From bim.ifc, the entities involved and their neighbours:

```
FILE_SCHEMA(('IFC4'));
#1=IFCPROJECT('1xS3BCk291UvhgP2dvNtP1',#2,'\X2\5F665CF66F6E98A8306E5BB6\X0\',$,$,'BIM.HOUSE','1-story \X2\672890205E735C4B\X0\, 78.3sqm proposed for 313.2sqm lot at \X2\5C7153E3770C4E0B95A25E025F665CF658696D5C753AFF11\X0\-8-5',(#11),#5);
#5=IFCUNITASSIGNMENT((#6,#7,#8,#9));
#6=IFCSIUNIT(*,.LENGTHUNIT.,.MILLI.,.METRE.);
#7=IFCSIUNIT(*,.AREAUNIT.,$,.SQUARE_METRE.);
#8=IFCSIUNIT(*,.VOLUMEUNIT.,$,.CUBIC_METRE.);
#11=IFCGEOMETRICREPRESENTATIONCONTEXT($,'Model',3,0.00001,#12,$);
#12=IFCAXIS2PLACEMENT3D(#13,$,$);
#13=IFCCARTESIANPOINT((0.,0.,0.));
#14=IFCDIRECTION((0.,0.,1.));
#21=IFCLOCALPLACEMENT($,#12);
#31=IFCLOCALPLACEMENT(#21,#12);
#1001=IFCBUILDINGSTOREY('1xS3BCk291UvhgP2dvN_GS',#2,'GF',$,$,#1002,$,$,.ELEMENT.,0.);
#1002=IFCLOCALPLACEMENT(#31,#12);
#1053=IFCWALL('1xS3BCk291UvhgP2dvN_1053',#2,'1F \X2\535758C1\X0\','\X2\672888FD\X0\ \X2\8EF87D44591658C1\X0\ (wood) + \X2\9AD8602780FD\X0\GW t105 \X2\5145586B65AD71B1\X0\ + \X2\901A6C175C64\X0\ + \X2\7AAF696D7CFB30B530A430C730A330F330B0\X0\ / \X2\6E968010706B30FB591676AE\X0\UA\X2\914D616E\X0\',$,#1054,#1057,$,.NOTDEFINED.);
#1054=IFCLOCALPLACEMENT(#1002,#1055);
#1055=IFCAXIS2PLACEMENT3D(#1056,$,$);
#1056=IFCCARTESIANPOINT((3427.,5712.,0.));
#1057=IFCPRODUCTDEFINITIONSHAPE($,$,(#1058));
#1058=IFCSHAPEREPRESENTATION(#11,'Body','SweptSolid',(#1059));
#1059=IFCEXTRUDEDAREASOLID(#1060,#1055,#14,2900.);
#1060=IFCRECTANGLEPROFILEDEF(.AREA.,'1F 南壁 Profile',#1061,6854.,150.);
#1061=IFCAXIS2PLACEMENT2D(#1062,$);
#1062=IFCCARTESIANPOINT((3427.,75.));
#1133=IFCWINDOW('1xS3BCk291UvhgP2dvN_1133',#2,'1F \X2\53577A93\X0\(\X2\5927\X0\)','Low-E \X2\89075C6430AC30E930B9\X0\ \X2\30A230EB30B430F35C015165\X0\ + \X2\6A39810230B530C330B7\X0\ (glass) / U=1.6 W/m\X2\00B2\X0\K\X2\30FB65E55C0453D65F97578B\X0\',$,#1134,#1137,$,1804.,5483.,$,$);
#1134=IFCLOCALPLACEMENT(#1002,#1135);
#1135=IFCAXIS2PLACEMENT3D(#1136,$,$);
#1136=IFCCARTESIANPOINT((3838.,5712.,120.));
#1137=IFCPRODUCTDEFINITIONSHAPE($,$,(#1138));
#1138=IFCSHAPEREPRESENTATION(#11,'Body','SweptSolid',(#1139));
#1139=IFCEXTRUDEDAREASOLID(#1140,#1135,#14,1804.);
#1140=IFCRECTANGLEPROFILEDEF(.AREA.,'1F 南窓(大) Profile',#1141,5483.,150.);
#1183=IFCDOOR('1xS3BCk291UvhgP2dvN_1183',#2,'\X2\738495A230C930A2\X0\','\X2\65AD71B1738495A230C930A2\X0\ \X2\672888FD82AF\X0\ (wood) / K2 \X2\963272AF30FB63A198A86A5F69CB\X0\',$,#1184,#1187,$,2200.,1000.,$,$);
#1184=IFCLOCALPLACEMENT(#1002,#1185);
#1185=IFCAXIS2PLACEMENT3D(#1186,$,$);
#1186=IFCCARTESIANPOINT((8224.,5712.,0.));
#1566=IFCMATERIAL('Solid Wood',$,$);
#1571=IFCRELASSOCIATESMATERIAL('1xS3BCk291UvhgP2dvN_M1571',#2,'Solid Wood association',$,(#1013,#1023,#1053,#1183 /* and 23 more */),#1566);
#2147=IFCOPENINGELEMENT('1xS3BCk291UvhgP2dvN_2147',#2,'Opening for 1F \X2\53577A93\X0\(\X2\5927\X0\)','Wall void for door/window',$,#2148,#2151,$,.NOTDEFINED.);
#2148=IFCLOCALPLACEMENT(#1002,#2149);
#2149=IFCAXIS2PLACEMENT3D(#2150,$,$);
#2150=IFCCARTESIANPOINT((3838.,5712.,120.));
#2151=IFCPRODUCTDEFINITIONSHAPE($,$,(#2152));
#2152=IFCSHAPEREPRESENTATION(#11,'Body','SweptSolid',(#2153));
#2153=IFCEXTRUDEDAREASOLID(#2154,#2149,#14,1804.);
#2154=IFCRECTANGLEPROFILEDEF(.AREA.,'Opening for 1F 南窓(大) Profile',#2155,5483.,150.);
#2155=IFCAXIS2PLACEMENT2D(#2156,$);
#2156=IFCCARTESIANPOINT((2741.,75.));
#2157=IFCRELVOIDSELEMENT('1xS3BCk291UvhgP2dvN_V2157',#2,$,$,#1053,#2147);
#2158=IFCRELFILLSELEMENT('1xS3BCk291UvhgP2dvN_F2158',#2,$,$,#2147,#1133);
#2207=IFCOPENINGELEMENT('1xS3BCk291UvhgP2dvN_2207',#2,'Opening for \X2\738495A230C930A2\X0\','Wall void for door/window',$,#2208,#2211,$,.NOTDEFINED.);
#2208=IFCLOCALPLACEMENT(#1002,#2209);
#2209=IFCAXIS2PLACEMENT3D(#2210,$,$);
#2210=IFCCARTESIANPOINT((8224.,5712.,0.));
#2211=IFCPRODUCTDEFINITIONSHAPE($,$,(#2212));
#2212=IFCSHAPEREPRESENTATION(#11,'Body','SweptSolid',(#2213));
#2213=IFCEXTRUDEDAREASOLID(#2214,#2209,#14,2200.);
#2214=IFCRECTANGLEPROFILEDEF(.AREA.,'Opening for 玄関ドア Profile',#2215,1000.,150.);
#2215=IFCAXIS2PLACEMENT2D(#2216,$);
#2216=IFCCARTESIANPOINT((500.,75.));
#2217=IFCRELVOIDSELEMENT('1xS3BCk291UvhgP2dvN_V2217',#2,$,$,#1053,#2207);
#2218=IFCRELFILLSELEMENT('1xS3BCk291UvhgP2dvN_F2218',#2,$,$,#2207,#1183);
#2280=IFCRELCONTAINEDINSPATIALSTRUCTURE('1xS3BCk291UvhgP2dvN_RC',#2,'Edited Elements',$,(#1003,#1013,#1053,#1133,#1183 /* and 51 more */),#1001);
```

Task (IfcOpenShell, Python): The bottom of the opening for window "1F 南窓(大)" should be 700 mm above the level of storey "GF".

```python
import numpy as np
import ifcopenshell
import ifcopenshell.api.geometry
import ifcopenshell.geom
import ifcopenshell.util.element
import ifcopenshell.util.placement
import ifcopenshell.util.shape
import ifcopenshell.util.unit

model = ifcopenshell.open("bim.ifc")
unit_scale = ifcopenshell.util.unit.calculate_unit_scale(model)

window = model.by_guid("1xS3BCk291UvhgP2dvN_1133")
opening = window.FillsVoids[0].RelatingOpeningElement
storey = ifcopenshell.util.element.get_container(window, ifc_class="IfcBuildingStorey")
level = ifcopenshell.util.placement.get_local_placement(storey.ObjectPlacement)[2, 3]

# The opening's origin need not be at the sill, so measure its lowest point.
shape = ifcopenshell.geom.create_shape(ifcopenshell.geom.settings(), opening)
bottom = ifcopenshell.util.shape.get_shape_bottom_elevation(shape, shape.geometry) / unit_scale
dz = level + 700.0 - bottom

shift = np.array([0.0, 0.0, dz])
# The window is not placed relative to its opening, so move both.
for product in (opening, window):
    matrix = ifcopenshell.util.placement.get_local_placement(product.ObjectPlacement)
    matrix[:3, 3] += shift
    ifcopenshell.api.geometry.edit_object_placement(model, product=product, matrix=matrix, is_si=False)

print(f"moved by {dz * unit_scale:+.3f} m")

model.write("bim_rev.ifc")
```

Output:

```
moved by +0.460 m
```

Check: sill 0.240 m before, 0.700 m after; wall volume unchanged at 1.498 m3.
